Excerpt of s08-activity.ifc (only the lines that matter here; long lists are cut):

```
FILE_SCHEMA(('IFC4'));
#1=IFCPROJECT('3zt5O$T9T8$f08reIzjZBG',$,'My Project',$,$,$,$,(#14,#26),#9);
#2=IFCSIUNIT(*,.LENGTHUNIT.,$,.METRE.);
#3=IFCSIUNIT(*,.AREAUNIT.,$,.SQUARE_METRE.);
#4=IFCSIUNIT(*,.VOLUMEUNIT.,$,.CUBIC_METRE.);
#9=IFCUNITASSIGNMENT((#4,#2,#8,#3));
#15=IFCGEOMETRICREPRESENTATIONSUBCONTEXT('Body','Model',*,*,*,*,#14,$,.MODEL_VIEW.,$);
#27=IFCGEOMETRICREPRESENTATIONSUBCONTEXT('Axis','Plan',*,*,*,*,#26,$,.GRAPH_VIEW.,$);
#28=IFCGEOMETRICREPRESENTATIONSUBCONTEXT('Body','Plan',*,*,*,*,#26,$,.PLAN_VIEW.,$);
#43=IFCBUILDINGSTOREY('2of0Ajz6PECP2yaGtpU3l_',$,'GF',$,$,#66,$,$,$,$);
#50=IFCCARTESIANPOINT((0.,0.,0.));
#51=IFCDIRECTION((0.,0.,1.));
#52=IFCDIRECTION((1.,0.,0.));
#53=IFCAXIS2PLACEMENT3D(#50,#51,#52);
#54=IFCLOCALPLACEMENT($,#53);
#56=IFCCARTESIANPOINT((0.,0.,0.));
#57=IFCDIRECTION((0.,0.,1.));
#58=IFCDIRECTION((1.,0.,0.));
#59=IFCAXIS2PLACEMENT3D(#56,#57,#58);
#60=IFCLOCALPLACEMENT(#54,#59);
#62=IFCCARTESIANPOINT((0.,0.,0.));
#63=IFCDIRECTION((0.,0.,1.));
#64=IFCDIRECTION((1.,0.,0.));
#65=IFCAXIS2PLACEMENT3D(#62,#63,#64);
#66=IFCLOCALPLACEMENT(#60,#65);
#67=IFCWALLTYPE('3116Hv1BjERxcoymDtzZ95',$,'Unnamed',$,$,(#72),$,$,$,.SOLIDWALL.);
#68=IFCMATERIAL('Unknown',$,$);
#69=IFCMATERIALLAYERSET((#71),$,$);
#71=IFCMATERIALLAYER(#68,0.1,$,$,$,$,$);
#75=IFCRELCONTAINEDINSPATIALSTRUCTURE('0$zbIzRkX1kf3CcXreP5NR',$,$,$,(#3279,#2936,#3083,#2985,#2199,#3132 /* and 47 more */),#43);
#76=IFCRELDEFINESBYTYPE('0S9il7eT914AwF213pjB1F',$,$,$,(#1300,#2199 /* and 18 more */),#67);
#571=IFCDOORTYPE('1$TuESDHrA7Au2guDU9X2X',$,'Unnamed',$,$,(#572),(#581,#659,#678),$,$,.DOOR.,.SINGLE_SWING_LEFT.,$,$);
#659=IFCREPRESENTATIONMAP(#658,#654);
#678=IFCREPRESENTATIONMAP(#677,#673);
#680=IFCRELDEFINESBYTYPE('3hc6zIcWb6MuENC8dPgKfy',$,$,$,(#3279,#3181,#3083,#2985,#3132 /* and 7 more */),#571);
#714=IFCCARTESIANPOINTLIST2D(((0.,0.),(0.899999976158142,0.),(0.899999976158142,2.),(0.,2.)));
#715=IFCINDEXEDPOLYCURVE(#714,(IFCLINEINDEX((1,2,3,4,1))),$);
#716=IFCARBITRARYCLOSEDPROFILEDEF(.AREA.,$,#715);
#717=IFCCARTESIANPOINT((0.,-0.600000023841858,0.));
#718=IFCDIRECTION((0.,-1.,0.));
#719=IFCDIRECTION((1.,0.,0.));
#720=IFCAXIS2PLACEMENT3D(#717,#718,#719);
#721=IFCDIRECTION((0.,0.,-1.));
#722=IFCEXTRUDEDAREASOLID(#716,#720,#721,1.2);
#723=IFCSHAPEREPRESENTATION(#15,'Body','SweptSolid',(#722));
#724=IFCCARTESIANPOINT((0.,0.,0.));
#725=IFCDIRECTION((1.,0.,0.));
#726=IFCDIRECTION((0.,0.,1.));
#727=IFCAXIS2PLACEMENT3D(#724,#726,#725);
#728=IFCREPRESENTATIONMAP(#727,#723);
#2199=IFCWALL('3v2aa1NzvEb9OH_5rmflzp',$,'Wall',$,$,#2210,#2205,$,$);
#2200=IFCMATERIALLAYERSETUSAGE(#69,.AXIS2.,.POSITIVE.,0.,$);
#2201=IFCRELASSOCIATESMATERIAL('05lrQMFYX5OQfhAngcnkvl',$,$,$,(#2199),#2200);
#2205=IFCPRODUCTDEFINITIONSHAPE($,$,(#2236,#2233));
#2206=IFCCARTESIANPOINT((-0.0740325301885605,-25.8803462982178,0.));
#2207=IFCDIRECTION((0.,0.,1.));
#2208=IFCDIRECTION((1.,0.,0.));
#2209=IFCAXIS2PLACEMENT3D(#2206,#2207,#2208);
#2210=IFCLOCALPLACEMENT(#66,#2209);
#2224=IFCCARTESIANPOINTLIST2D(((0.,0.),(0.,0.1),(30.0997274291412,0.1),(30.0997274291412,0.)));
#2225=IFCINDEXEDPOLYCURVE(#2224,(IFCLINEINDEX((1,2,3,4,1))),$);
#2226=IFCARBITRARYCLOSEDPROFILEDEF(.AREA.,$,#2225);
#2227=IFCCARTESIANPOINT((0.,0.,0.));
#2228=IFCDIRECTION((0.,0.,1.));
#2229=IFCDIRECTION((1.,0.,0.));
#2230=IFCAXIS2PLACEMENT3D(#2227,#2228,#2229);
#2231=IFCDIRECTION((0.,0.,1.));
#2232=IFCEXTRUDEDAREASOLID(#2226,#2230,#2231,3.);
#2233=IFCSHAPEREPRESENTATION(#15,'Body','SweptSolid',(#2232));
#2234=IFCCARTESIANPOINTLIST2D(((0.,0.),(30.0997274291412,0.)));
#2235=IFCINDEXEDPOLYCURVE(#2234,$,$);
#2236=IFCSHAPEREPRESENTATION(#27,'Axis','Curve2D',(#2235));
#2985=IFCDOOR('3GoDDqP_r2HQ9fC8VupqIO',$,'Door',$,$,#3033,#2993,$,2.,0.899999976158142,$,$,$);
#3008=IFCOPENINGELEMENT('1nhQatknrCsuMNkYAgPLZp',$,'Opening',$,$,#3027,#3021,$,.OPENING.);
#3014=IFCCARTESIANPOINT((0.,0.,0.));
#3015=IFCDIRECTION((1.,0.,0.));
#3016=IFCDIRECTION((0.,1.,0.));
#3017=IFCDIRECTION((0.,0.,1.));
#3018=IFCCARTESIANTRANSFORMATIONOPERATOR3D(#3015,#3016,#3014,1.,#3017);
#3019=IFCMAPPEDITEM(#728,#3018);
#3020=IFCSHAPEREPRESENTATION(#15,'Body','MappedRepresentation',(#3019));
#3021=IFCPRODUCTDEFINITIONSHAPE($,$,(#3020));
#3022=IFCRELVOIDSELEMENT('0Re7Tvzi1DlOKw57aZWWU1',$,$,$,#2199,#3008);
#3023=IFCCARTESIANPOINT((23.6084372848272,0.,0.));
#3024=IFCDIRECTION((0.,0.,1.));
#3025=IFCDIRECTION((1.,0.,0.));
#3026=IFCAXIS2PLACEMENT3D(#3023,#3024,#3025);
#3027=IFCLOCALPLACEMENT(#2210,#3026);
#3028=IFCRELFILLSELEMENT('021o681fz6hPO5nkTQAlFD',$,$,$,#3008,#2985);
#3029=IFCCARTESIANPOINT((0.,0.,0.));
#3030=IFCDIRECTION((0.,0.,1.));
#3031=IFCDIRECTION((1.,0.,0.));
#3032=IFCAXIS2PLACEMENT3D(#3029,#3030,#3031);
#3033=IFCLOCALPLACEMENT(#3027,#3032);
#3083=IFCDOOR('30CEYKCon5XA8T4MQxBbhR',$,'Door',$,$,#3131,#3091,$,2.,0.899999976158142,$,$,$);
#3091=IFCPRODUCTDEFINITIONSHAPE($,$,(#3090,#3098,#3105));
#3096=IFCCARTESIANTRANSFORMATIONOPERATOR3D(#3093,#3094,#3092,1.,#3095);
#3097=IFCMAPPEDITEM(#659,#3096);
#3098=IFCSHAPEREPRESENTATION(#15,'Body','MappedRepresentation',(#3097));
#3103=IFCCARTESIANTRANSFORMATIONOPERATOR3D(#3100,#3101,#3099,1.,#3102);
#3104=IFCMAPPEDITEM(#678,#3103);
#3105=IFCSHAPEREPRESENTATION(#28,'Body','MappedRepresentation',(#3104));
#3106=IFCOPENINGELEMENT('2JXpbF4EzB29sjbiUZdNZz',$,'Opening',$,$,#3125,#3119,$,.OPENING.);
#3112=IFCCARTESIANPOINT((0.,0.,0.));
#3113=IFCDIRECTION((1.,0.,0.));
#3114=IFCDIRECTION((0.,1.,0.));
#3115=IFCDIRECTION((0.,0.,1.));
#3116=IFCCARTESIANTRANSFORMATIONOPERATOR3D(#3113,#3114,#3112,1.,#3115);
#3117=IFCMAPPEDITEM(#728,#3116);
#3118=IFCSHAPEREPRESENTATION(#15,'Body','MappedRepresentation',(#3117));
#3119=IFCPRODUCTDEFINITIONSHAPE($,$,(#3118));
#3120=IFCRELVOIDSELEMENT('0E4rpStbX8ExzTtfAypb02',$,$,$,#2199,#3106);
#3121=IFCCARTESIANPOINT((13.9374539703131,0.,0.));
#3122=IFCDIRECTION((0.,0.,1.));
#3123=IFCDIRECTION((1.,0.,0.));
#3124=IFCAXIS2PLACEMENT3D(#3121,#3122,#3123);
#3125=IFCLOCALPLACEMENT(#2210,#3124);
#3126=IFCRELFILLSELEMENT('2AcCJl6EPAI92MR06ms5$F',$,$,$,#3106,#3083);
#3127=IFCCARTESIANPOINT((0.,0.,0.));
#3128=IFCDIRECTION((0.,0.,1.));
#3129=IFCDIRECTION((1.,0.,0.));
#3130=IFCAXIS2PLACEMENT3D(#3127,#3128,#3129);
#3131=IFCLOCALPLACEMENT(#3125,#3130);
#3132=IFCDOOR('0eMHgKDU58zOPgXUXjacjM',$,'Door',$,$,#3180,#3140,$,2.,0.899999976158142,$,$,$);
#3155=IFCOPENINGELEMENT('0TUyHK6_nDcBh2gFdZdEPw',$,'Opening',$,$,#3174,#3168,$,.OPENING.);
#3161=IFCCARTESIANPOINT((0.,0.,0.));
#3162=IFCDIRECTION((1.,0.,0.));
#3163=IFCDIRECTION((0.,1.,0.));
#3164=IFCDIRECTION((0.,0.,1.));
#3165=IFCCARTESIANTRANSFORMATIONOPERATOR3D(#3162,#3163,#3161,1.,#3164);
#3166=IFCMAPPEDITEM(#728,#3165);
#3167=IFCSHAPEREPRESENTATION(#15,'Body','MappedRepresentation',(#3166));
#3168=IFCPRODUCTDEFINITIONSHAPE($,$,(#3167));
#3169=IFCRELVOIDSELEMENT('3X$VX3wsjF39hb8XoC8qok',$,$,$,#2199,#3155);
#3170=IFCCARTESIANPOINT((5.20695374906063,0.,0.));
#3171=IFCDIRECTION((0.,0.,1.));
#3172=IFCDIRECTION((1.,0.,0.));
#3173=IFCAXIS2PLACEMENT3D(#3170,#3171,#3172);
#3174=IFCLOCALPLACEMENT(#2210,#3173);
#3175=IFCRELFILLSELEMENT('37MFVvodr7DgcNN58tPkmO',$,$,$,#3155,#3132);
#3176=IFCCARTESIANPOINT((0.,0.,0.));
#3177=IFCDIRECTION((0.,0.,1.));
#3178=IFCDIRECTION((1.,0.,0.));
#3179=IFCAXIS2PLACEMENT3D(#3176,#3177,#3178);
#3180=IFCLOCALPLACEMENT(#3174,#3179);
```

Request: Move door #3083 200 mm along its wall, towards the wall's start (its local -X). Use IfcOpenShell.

```python
import ifcopenshell
import ifcopenshell.api.geometry
import ifcopenshell.util.placement
import ifcopenshell.util.unit

model = ifcopenshell.open("s08-activity.ifc")
unit_scale = ifcopenshell.util.unit.calculate_unit_scale(model)

door = model.by_id(3083)
opening = door.FillsVoids[0].RelatingOpeningElement
wall = opening.VoidsElements[0].RelatingBuildingElement

wall_matrix = ifcopenshell.util.placement.get_local_placement(wall.ObjectPlacement)
shift = wall_matrix[:3, 0] * -0.2 / unit_scale
before = ifcopenshell.util.placement.get_local_placement(door.ObjectPlacement)[:3, 3].copy()

# The door is placed relative to its opening, so it follows when the opening moves.
matrix = ifcopenshell.util.placement.get_local_placement(opening.ObjectPlacement)
matrix[:3, 3] += shift
ifcopenshell.api.geometry.edit_object_placement(
    model, product=opening, matrix=matrix, is_si=False, should_transform_children=True
)

after = ifcopenshell.util.placement.get_local_placement(door.ObjectPlacement)[:3, 3]
print("door moved by", (after - before).round(3) + 0.0)

model.write("s08-activity_rev.ifc")
```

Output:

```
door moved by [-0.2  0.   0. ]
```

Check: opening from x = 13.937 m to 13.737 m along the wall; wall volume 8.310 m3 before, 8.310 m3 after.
